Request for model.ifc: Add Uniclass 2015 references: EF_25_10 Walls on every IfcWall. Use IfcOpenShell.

First a look at what the model holds.

```python
import ifcopenshell

model = ifcopenshell.open("model.ifc")
print(model.schema)
print("classifications:", [c.Name for c in model.by_type("IfcClassification")])
for ifc_class in ("IfcDoor", "IfcRoof", "IfcStair", "IfcWall", "IfcWindow"):
    print(ifc_class, len(model.by_type(ifc_class)))
```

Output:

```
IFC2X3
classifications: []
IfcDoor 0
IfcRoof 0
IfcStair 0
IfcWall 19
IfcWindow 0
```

```python
import ifcopenshell
import ifcopenshell.api.classification

model = ifcopenshell.open("model.ifc")

# IFC2X3 requires Source and Edition and has no link from the project to the system.
system = model.create_entity("IfcClassification", Source="NBS", Edition="2015", Name="Uniclass 2015")

codes = {
    "IfcWall": ("EF_25_10", "Walls"),
}
for ifc_class, (code, name) in codes.items():
    products = model.by_type(ifc_class)
    ifcopenshell.api.classification.add_reference(
        model, products=products, classification=system, identification=code, name=name
    )
    print(code, len(products))

model.write("model_v2.ifc")
```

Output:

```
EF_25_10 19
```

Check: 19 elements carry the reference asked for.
